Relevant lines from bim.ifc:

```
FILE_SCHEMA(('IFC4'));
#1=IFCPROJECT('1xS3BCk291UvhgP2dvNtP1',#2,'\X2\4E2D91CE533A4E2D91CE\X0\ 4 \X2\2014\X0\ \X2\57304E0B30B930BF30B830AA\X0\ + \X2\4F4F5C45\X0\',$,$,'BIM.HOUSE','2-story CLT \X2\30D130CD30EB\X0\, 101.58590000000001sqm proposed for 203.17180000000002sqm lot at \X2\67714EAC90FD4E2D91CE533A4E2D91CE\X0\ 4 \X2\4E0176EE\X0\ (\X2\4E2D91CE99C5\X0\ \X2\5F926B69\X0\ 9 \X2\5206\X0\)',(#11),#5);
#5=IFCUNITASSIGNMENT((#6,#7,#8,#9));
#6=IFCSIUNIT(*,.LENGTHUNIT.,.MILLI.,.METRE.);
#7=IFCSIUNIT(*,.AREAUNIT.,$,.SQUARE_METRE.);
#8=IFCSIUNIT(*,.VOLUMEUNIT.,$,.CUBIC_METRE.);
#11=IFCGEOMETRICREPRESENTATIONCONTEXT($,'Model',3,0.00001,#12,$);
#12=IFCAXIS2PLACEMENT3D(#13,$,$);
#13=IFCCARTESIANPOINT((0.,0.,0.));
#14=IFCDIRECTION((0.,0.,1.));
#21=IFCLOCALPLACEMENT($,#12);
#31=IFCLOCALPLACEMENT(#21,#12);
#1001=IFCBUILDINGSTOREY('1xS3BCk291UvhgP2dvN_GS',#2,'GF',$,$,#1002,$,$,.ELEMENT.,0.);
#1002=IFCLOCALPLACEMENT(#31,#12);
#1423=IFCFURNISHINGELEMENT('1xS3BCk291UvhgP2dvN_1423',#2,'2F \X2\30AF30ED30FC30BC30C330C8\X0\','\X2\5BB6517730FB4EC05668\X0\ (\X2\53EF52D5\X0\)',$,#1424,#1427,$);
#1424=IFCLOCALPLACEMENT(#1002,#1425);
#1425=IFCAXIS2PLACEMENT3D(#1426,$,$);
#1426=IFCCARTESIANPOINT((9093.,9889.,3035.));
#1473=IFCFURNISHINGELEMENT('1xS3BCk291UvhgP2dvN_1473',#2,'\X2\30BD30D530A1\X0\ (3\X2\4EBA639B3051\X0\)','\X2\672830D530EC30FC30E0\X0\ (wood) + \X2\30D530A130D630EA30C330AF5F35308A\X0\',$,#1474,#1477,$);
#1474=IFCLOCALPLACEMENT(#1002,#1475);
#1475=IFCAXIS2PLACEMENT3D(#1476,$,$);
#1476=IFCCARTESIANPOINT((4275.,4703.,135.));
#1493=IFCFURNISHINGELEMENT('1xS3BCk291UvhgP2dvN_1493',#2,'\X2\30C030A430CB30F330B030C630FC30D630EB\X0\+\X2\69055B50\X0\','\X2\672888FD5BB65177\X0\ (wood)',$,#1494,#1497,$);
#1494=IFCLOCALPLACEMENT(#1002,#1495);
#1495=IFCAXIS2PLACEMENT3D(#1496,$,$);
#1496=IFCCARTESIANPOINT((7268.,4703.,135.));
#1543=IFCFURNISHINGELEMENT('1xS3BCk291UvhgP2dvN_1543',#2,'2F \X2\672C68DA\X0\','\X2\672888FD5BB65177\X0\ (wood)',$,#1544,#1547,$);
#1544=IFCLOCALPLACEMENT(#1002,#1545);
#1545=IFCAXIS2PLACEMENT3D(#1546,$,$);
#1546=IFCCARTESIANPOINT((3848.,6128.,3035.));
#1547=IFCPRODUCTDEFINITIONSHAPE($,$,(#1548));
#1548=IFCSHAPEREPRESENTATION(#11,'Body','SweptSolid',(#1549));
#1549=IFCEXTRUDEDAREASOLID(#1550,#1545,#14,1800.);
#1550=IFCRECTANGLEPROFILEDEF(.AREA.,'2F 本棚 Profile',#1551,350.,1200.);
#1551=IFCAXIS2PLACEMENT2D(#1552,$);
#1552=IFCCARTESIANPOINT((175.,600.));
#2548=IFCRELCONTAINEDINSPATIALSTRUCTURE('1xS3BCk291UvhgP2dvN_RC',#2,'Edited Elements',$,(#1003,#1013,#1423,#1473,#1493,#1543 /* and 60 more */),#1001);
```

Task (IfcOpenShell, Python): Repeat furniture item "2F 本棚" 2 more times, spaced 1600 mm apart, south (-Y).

```python
import numpy as np
import ifcopenshell
import ifcopenshell.api.geometry
import ifcopenshell.api.root
import ifcopenshell.util.element
import ifcopenshell.util.placement

model = ifcopenshell.open("bim.ifc")


def reuse_history(source, copy):
    """copy_class also copies each property set's owner history, people and application; keep the originals."""
    for rel in copy.IsDefinedBy:
        if rel.is_a("IfcRelDefinesByProperties") and (history := rel.RelatingPropertyDefinition.OwnerHistory):
            rel.RelatingPropertyDefinition.OwnerHistory = source.OwnerHistory
            ifcopenshell.util.element.remove_deep2(model, history)


source = model.by_guid("1xS3BCk291UvhgP2dvN_1543")
base = ifcopenshell.util.placement.get_local_placement(source.ObjectPlacement)
step = np.array([0.0, -1.0, 0.0]) * 1600.0

for i in range(1, 3):
    copy = ifcopenshell.api.root.copy_class(model, product=source)
    copy.Representation = ifcopenshell.util.element.copy_deep(
        model, source.Representation, exclude=["IfcGeometricRepresentationContext", "IfcRepresentationMap"]
    )
    reuse_history(source, copy)
    matrix = base.copy()
    matrix[:3, 3] += i * step
    print("added at", matrix[:3, 3].round(3) + 0.0)
    ifcopenshell.api.geometry.edit_object_placement(model, product=copy, matrix=matrix, is_si=False)

model.write("bim_v2.ifc")
```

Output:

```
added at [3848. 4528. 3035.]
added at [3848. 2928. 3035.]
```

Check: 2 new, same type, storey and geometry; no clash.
